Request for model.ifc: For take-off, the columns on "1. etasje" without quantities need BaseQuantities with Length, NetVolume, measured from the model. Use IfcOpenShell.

First a look at what the model holds.

```python
import ifcopenshell
import ifcopenshell.util.element
import ifcopenshell.util.unit

model = ifcopenshell.open("model.ifc")
print(model.schema)
for unit_type in ("LENGTHUNIT", "AREAUNIT", "VOLUMEUNIT"):
    print(unit_type, ifcopenshell.util.unit.calculate_unit_scale(model, unit_type))
storey = next(s for s in model.by_type("IfcBuildingStorey") if s.Name == "1. etasje")
columns = [e for e in ifcopenshell.util.element.get_decomposition(storey) if e.is_a("IfcColumn")]
for e in sorted(columns, key=lambda e: e.id()):
    print(e.id(), e.is_a(), e.Name, list(ifcopenshell.util.element.get_psets(e, qtos_only=True)), sep=" | ")
```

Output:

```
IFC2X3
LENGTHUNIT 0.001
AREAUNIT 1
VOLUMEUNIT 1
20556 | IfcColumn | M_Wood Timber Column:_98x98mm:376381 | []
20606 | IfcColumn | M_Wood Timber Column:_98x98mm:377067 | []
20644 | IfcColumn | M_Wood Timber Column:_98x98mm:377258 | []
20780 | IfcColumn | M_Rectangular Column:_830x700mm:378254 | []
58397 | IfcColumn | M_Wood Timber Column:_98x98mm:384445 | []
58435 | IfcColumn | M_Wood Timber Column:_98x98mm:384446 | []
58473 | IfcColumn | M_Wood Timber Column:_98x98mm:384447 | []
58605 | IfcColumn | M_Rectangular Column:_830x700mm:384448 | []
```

```python
import ifcopenshell
import ifcopenshell.api.pset
import ifcopenshell.geom
import ifcopenshell.util.element
import ifcopenshell.util.shape
import ifcopenshell.util.unit

model = ifcopenshell.open("model.ifc")
unit_scale = ifcopenshell.util.unit.calculate_unit_scale(model)
volume_scale = ifcopenshell.util.unit.calculate_unit_scale(model, "VOLUMEUNIT")
settings = ifcopenshell.geom.settings()

storey = next(s for s in model.by_type("IfcBuildingStorey") if s.Name == "1. etasje")
columns = [e for e in ifcopenshell.util.element.get_decomposition(storey) if e.is_a("IfcColumn")]

for e in sorted(columns, key=lambda e: e.id()):
    if ifcopenshell.util.element.get_psets(e, qtos_only=True, should_inherit=False):
        continue
    # Geometry comes back in metres, in the element's own axes.
    shape = ifcopenshell.geom.create_shape(settings, e)
    values = {
        "Length": ifcopenshell.util.shape.get_z(shape.geometry) / unit_scale,
        "NetVolume": ifcopenshell.util.shape.get_volume(shape.geometry) / volume_scale,
    }
    qto = ifcopenshell.api.pset.add_qto(model, product=e, name="BaseQuantities")
    ifcopenshell.api.pset.edit_qto(model, qto=qto, properties=values)
    print(e.id(), {k: round(v, 3) for k, v in values.items()})

model.write("model_updated.ifc")
```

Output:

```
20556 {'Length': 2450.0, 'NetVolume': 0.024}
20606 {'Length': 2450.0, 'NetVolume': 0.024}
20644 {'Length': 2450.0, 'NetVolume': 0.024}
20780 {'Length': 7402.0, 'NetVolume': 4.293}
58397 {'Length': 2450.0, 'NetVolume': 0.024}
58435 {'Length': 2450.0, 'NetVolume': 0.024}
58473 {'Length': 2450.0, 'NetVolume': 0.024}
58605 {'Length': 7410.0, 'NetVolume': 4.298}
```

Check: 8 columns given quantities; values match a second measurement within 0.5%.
